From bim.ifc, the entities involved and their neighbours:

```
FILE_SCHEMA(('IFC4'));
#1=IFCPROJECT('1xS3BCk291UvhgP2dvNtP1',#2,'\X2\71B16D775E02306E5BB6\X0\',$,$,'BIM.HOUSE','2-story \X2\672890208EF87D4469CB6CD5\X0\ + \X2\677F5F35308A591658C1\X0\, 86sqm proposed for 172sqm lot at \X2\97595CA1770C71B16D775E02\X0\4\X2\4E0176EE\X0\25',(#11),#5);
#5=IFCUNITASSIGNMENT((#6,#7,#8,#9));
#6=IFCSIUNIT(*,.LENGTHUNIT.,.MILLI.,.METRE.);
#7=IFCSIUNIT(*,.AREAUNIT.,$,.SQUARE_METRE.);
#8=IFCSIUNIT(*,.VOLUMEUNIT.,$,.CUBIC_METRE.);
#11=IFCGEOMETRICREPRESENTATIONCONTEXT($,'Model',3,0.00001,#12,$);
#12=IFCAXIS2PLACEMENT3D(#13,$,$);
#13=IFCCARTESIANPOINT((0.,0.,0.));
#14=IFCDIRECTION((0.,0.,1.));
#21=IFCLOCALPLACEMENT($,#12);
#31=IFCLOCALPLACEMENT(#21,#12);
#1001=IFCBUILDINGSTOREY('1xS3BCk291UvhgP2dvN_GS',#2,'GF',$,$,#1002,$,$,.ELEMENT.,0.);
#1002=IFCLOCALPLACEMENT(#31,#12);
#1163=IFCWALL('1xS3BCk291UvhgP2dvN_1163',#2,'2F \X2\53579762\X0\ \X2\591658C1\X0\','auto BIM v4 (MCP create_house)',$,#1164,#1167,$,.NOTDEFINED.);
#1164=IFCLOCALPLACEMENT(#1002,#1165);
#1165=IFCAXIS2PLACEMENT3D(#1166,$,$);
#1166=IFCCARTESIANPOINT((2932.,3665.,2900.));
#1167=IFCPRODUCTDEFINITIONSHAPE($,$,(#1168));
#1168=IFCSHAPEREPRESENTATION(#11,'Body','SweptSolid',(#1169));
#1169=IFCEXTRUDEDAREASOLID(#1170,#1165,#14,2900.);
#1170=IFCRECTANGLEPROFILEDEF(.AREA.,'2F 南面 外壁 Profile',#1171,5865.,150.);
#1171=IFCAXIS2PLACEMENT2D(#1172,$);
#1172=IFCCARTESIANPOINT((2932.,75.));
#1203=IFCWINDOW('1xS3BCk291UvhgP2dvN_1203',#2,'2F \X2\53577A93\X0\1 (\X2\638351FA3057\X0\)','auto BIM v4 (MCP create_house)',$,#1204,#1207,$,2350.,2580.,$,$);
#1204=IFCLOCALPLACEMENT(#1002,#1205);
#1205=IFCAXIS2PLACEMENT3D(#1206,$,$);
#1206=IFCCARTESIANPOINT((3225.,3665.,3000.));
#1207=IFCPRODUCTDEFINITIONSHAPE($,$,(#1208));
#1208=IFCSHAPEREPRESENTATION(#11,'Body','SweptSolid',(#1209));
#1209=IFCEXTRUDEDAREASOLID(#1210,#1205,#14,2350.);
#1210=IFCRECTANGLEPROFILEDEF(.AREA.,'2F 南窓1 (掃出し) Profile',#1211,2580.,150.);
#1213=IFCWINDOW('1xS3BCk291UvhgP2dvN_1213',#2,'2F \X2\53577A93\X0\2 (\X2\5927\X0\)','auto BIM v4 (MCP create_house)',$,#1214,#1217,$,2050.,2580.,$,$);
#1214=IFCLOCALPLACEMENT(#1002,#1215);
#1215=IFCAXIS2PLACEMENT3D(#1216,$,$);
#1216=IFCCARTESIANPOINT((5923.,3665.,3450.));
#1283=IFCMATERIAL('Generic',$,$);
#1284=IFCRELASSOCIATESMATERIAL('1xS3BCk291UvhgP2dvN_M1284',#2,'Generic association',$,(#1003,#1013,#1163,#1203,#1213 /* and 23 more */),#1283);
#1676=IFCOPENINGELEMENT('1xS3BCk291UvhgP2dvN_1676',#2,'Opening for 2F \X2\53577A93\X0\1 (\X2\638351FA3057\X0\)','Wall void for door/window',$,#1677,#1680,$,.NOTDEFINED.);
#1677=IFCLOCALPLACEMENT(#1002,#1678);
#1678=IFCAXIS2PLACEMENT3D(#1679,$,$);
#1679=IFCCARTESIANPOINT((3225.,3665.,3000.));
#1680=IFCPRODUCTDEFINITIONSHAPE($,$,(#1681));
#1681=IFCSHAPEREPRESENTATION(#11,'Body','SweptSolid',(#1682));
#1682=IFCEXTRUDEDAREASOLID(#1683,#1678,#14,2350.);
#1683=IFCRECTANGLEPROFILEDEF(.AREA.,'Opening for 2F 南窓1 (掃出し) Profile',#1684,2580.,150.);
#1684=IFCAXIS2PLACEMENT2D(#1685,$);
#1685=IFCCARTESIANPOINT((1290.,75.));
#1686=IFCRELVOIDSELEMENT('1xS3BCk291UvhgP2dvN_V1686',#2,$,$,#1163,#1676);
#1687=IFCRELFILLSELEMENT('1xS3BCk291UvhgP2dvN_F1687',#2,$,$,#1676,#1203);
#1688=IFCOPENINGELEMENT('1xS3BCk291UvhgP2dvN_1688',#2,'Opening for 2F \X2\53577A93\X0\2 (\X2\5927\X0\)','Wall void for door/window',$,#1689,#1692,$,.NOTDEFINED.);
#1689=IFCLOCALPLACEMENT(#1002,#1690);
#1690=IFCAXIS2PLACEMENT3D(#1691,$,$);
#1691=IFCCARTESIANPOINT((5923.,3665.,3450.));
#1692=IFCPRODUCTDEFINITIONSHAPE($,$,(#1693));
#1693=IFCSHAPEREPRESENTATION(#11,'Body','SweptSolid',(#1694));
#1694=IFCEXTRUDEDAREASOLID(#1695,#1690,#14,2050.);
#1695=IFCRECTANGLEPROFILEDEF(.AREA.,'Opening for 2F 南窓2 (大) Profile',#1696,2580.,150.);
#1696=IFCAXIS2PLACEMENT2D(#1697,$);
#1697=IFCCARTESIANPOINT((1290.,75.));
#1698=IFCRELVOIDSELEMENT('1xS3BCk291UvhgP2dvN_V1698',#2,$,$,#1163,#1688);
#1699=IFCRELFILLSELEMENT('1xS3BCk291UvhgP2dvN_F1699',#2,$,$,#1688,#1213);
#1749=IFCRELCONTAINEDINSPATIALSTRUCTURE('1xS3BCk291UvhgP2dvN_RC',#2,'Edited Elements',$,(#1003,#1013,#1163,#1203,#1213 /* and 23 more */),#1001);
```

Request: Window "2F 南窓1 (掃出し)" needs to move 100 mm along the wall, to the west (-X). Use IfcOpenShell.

```python
import ifcopenshell
import ifcopenshell.api.geometry
import ifcopenshell.util.placement

model = ifcopenshell.open("bim.ifc")

window = model.by_id(1203)
opening = window.FillsVoids[0].RelatingOpeningElement
wall = opening.VoidsElements[0].RelatingBuildingElement

wall_matrix = ifcopenshell.util.placement.get_local_placement(wall.ObjectPlacement)
shift = wall_matrix[:3, 0] * -100.0
before = ifcopenshell.util.placement.get_local_placement(window.ObjectPlacement)[:3, 3].copy()

# The window is not placed relative to its opening, so move both.
for product in (opening, window):
    matrix = ifcopenshell.util.placement.get_local_placement(product.ObjectPlacement)
    matrix[:3, 3] += shift
    ifcopenshell.api.geometry.edit_object_placement(model, product=product, matrix=matrix, is_si=False)

after = ifcopenshell.util.placement.get_local_placement(window.ObjectPlacement)[:3, 3]
print("window moved by", (after - before).round(3) + 0.0)

model.write("bim_updated.ifc")
```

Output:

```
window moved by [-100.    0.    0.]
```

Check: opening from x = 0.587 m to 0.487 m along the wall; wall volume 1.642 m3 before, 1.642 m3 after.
